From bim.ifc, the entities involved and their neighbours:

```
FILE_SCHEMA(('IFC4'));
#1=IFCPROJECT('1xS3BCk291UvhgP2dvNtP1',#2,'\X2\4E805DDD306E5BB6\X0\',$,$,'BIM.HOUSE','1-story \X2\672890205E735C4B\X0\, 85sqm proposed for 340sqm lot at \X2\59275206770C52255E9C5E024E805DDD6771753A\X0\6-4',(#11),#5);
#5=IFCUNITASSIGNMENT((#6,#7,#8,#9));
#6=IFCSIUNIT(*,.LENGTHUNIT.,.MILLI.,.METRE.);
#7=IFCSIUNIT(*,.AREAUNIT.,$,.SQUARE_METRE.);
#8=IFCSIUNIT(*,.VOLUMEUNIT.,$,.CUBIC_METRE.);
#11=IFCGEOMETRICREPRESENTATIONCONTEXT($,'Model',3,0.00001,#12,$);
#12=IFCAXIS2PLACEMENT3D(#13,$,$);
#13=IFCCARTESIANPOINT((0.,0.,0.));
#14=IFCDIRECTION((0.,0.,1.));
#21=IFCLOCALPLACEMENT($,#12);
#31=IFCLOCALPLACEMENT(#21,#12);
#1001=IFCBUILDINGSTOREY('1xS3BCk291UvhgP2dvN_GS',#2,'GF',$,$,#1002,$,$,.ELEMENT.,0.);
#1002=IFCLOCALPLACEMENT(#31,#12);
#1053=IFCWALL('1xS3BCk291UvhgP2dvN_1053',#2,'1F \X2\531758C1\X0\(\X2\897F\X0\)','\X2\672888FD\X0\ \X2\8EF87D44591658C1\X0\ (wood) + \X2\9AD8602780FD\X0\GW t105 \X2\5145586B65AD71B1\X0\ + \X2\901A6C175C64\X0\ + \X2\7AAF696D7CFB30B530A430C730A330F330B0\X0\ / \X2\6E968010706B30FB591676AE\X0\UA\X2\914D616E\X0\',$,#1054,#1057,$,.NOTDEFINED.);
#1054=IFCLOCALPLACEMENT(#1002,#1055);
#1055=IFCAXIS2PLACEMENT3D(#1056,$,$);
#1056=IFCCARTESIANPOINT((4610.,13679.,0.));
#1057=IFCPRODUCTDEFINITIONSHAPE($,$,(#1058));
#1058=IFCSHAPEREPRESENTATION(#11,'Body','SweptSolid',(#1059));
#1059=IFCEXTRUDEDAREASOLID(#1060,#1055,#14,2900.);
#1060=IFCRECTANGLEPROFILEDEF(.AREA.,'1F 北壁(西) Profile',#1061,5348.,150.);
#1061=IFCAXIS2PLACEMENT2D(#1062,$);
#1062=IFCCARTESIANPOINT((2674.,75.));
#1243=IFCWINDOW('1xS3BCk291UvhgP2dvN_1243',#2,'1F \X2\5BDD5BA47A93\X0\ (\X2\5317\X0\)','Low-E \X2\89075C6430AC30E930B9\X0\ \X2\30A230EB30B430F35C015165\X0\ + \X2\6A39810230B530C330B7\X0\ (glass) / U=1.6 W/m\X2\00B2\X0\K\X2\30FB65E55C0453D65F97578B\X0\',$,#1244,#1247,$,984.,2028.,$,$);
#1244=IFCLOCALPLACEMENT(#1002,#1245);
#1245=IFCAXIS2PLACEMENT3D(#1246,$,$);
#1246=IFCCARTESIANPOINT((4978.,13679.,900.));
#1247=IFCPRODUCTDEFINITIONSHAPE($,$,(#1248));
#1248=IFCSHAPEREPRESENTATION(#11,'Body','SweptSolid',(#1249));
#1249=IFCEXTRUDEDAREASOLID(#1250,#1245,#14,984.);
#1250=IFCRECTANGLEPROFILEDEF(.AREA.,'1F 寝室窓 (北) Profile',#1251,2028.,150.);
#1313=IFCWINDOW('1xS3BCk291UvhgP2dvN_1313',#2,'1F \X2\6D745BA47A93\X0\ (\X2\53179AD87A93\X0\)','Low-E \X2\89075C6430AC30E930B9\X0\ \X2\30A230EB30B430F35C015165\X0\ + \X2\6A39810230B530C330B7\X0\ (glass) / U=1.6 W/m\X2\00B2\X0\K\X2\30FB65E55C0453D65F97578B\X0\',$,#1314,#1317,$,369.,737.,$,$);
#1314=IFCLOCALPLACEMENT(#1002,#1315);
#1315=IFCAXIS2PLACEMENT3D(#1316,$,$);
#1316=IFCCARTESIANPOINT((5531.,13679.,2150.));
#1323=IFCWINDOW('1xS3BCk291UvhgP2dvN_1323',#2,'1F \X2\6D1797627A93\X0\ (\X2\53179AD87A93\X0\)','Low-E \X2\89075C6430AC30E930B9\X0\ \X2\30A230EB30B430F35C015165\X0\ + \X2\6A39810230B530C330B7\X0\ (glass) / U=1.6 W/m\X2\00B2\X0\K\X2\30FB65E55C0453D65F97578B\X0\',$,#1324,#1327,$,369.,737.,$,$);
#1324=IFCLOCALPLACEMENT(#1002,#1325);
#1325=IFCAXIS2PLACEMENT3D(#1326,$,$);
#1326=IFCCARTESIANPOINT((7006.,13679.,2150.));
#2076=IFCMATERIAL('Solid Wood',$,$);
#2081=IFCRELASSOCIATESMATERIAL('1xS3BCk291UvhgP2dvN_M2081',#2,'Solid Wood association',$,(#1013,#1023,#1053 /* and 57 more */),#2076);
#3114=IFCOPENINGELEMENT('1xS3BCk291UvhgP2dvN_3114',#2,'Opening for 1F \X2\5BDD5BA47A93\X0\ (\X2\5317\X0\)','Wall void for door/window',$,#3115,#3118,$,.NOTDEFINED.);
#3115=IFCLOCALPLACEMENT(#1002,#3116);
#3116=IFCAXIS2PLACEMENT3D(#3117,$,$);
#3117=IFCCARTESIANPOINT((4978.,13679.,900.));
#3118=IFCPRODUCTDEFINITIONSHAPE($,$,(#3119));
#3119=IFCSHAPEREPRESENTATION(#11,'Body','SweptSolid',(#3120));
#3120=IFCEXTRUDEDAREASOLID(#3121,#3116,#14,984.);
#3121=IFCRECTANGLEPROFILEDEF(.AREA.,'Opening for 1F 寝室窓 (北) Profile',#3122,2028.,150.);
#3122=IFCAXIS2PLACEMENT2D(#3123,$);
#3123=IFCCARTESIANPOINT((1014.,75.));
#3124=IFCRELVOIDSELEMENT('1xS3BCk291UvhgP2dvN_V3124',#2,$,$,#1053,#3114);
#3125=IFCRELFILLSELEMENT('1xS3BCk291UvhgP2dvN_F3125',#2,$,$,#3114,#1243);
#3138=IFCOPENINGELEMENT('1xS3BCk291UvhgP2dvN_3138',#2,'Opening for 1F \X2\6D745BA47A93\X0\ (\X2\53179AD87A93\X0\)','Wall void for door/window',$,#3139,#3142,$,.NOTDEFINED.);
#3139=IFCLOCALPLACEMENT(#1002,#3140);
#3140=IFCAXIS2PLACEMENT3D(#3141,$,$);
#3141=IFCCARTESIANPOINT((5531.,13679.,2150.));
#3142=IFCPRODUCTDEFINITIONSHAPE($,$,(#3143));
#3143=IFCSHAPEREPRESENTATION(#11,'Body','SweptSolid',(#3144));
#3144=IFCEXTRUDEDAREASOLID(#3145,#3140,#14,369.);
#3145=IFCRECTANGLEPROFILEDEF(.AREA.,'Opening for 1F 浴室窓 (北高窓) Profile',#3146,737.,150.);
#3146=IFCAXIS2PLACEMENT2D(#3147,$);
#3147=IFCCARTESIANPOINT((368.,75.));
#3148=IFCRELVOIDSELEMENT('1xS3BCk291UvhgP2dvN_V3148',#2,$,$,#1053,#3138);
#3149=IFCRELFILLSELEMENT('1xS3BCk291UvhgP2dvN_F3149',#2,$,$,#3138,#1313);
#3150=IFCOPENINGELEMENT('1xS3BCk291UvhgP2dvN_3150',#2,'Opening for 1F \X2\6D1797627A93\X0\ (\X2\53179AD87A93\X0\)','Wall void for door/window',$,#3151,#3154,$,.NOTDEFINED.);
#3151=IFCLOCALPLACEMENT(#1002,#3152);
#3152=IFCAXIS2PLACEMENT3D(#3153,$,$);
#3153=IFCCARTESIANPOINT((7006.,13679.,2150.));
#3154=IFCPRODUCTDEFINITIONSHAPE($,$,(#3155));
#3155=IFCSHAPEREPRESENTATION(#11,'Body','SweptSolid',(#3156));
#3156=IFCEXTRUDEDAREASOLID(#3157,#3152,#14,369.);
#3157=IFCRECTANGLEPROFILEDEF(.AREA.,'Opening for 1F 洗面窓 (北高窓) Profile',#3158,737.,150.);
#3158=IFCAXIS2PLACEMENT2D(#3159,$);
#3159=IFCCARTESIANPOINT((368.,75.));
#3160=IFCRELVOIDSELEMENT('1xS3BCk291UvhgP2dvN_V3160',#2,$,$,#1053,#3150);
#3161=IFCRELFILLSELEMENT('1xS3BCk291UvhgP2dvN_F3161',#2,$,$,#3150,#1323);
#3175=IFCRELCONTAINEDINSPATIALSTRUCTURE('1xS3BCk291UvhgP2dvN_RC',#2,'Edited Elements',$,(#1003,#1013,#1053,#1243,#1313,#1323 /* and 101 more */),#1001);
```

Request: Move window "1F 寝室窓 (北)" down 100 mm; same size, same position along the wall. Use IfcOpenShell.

```python
import numpy as np
import ifcopenshell
import ifcopenshell.api.geometry
import ifcopenshell.util.placement
import ifcopenshell.util.unit

model = ifcopenshell.open("bim.ifc")
unit_scale = ifcopenshell.util.unit.calculate_unit_scale(model)

window = model.by_id(1243)
opening = window.FillsVoids[0].RelatingOpeningElement
dz = -0.1 / unit_scale

shift = np.array([0.0, 0.0, dz])
# The window is not placed relative to its opening, so move both.
for product in (opening, window):
    matrix = ifcopenshell.util.placement.get_local_placement(product.ObjectPlacement)
    matrix[:3, 3] += shift
    ifcopenshell.api.geometry.edit_object_placement(model, product=product, matrix=matrix, is_si=False)

print(f"moved by {dz * unit_scale:+.3f} m")

model.write("bim_rev.ifc")
```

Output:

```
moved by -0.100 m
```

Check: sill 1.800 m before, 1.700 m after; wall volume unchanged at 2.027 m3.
